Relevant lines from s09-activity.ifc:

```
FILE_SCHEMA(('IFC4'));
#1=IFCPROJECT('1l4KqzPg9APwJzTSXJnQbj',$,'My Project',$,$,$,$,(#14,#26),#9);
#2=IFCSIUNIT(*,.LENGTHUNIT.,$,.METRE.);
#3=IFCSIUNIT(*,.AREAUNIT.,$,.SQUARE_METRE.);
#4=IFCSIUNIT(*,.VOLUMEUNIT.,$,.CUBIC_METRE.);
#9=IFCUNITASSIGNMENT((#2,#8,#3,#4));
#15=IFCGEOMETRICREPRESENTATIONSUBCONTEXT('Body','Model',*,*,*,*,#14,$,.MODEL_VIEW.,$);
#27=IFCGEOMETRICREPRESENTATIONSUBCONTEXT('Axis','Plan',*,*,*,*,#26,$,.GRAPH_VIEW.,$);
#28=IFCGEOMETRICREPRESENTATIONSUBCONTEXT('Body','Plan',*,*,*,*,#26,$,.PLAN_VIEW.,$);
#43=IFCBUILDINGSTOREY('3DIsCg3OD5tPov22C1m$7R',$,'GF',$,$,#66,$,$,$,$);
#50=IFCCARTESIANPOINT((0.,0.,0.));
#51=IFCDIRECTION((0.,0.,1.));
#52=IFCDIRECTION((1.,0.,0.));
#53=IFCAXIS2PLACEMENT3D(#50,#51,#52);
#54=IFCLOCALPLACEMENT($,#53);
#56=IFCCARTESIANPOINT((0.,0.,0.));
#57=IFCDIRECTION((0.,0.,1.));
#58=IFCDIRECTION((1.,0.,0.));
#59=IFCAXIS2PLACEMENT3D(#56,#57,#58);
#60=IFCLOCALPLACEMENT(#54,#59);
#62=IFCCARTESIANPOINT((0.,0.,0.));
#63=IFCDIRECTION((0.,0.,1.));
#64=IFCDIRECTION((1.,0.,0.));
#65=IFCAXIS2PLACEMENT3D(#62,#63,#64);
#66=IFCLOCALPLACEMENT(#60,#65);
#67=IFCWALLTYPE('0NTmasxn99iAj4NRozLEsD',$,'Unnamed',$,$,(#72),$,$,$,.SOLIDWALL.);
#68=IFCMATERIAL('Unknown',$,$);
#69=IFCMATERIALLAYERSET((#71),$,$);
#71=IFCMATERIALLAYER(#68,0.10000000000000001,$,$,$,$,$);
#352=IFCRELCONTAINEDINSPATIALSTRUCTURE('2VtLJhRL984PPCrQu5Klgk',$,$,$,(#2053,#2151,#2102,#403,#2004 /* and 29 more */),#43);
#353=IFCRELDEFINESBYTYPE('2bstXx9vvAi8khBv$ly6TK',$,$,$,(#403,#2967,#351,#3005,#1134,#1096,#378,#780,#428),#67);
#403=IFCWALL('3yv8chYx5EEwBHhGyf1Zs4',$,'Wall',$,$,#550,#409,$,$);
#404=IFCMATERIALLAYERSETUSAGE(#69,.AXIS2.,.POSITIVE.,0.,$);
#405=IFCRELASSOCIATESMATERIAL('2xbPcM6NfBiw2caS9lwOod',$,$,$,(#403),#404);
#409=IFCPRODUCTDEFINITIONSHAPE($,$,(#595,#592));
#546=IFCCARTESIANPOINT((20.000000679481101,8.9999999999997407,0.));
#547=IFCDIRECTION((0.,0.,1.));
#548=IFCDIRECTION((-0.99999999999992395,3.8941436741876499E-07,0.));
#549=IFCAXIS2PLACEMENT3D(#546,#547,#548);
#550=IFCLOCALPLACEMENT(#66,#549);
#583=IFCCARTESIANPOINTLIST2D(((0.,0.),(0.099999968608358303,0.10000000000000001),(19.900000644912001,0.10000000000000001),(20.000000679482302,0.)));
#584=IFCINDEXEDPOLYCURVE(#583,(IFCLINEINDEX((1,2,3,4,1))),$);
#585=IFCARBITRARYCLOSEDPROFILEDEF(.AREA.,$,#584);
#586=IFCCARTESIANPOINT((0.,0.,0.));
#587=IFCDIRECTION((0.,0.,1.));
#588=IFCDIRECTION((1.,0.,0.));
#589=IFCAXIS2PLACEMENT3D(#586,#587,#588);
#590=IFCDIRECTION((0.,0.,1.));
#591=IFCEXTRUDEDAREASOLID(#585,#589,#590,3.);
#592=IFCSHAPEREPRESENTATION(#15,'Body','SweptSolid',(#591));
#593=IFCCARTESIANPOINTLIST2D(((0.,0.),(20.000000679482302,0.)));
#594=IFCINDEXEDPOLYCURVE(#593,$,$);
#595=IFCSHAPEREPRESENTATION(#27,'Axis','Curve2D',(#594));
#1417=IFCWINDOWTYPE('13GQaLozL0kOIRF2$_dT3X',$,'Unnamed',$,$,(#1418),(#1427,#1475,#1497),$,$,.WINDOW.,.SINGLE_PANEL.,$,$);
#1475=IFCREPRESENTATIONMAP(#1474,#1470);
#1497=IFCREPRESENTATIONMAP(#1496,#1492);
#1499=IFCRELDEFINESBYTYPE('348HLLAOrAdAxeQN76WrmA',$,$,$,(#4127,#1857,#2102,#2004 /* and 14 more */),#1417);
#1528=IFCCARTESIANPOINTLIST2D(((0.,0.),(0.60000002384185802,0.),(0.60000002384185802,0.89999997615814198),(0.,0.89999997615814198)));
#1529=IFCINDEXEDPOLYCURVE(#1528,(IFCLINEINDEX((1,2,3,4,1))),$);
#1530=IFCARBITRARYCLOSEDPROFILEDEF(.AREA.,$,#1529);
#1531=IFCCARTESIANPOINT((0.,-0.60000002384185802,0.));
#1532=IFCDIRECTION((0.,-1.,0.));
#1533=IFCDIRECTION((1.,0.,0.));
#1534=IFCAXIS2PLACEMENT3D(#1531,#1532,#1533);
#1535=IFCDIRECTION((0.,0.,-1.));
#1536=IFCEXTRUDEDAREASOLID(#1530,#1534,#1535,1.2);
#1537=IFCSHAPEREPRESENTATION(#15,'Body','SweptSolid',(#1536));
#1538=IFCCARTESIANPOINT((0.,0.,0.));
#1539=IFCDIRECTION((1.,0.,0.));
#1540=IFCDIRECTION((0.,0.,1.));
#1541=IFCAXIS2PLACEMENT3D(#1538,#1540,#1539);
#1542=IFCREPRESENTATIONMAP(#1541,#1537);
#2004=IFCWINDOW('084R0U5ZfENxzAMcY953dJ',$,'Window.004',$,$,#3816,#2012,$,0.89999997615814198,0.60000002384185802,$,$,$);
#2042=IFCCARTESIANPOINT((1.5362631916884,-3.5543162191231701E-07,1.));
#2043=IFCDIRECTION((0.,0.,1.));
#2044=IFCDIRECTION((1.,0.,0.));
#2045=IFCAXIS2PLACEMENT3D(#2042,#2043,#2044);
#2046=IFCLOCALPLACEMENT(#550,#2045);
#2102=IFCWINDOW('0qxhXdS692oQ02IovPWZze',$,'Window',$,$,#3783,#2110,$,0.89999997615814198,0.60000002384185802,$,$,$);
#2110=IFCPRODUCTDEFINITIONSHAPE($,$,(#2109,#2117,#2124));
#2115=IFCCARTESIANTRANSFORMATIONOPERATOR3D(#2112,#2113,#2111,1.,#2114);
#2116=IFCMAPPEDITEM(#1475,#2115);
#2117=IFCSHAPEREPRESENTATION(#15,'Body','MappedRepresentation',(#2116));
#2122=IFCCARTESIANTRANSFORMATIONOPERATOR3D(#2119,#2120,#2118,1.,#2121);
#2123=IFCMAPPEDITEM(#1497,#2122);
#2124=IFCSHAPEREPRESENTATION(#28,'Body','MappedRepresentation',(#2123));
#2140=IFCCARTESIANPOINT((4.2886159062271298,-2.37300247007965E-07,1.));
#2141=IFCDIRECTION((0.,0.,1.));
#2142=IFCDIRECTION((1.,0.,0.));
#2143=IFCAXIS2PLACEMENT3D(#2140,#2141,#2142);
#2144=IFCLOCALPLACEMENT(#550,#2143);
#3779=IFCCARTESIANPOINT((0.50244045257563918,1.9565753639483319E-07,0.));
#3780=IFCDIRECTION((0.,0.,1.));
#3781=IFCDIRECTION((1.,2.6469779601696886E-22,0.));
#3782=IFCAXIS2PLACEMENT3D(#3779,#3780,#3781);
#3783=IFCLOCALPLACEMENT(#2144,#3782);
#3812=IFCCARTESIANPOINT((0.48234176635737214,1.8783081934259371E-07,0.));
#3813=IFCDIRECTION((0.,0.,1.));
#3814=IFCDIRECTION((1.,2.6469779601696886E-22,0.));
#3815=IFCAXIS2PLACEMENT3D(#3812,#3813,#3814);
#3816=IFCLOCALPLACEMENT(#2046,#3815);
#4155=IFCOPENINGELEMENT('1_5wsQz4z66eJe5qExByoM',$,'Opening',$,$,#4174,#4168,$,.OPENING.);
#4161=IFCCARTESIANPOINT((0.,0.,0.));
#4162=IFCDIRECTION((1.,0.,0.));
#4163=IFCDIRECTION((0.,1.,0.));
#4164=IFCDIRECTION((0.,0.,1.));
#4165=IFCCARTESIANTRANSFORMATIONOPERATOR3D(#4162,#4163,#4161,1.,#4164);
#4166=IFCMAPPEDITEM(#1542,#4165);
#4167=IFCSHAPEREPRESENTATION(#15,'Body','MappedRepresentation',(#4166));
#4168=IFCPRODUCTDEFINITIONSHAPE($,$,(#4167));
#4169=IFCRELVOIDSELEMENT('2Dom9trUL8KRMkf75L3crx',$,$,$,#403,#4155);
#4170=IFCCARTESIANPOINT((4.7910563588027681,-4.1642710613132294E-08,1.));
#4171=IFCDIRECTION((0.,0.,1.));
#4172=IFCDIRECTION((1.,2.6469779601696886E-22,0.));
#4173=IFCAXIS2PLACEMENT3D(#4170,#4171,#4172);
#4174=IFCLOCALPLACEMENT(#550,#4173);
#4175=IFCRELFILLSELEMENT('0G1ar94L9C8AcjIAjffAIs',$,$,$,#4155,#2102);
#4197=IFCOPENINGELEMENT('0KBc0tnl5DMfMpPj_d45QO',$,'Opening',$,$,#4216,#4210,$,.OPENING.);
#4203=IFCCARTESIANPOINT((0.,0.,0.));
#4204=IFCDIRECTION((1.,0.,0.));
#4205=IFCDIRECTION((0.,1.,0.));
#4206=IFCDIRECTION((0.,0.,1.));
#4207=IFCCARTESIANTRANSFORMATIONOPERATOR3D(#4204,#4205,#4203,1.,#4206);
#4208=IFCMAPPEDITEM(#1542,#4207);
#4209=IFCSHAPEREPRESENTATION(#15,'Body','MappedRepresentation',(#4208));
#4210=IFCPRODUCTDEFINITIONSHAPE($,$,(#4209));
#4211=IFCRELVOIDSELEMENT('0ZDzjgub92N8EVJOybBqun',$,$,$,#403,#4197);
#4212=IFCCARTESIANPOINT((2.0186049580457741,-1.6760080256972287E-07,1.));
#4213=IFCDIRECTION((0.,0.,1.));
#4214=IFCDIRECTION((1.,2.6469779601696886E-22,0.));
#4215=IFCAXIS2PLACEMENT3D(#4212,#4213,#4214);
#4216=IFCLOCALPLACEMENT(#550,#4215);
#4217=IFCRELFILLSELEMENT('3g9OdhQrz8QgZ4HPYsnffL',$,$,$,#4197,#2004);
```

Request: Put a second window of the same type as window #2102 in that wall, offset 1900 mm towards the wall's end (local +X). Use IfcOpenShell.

```python
import ifcopenshell
import ifcopenshell.api.feature
import ifcopenshell.api.geometry
import ifcopenshell.api.root
import ifcopenshell.geom
import ifcopenshell.util.element
import ifcopenshell.util.placement
import ifcopenshell.util.shape
import ifcopenshell.util.unit

model = ifcopenshell.open("s09-activity.ifc")
unit_scale = ifcopenshell.util.unit.calculate_unit_scale(model)
settings = ifcopenshell.geom.settings()


def volume(element):
    """Net volume in cubic metres, openings subtracted."""
    shape = ifcopenshell.geom.create_shape(settings, element)
    return ifcopenshell.util.shape.get_volume(shape.geometry)


window = model.by_guid("0qxhXdS692oQ02IovPWZze")
opening = window.FillsVoids[0].RelatingOpeningElement
wall = opening.VoidsElements[0].RelatingBuildingElement
before = volume(wall)
shift = ifcopenshell.util.placement.get_local_placement(wall.ObjectPlacement)[:3, 0] * 1.9 / unit_scale

# copy_class copies the void relationship, type, container and properties, but no geometry.
new_opening = ifcopenshell.api.root.copy_class(model, product=opening)
new_opening.Representation = ifcopenshell.util.element.copy_deep(
    model, opening.Representation, exclude=["IfcGeometricRepresentationContext", "IfcRepresentationMap"]
)
new_window = ifcopenshell.api.root.copy_class(model, product=window)
new_window.Representation = ifcopenshell.util.element.copy_deep(
    model, window.Representation, exclude=["IfcGeometricRepresentationContext", "IfcRepresentationMap"]
)
ifcopenshell.api.feature.add_filling(model, opening=new_opening, element=new_window)

for old, new in ((opening, new_opening), (window, new_window)):
    matrix = ifcopenshell.util.placement.get_local_placement(old.ObjectPlacement)
    matrix[:3, 3] += shift
    ifcopenshell.api.geometry.edit_object_placement(model, product=new, matrix=matrix, is_si=False)

after = volume(wall)

print(f"wall volume {before:.3f} -> {after:.3f} m3")

model.write("s09-activity_updated.ifc")
```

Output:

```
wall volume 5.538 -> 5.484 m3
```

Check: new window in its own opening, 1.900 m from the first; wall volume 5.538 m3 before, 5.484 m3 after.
